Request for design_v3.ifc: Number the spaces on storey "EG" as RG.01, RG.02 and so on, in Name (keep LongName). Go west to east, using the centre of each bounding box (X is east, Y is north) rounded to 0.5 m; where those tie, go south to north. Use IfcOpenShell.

First a look at what the model holds.

```python
import ifcopenshell
import ifcopenshell.util.element
import ifcopenshell.util.placement

model = ifcopenshell.open("design_v3.ifc")
print(model.schema)
storey = next(s for s in model.by_type("IfcBuildingStorey") if s.Name == "EG")
spaces = [e for e in ifcopenshell.util.element.get_decomposition(storey) if e.is_a("IfcSpace")]
for e in sorted(spaces, key=lambda e: e.id()):
    origin = ifcopenshell.util.placement.get_local_placement(e.ObjectPlacement)[:3, 3]
    print(e.id(), e.Name, e.LongName, origin.round(2) + 0.0, sep=" | ")
```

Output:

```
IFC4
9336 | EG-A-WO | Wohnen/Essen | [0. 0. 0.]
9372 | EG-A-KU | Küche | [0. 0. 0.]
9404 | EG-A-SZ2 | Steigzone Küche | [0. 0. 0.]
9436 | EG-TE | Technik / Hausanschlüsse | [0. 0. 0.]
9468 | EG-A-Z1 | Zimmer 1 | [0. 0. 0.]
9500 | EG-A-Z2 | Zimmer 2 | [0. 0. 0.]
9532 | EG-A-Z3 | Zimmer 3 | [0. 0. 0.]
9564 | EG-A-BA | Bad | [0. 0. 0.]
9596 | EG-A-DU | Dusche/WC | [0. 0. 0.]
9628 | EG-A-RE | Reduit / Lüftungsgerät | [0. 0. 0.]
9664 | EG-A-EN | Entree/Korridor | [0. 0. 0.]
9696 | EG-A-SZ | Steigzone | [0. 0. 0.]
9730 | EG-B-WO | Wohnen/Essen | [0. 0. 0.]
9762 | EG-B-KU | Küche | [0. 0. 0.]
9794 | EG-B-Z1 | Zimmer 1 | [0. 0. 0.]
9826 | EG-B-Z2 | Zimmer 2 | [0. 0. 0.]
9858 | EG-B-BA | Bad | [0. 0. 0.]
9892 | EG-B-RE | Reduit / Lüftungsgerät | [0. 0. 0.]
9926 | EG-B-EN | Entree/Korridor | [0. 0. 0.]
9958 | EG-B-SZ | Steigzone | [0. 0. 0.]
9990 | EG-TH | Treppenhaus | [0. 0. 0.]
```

```python
import ifcopenshell
import ifcopenshell.geom
import ifcopenshell.util.element
import ifcopenshell.util.shape

model = ifcopenshell.open("design_v3.ifc")
settings = ifcopenshell.geom.settings()
settings.set("use-world-coords", True)


def centre(element):
    shape = ifcopenshell.geom.create_shape(settings, element)
    return ifcopenshell.util.shape.get_bbox_centroid(shape.geometry)


storey = next(s for s in model.by_type("IfcBuildingStorey") if s.Name == "EG")
spaces = [e for e in ifcopenshell.util.element.get_decomposition(storey) if e.is_a("IfcSpace")]

# Insertion points can sit at a corner or the storey origin, so sort by the geometry (in metres).
centres = {e: centre(e) for e in spaces}
spaces.sort(key=lambda e: (round(centres[e][0] / 0.5), centres[e][1]))

for i, e in enumerate(spaces, start=1):
    number = f"RG.{i:02d}"
    e.Name = number
    print(e.id(), number)

model.write("design_v3_v2.ifc")
```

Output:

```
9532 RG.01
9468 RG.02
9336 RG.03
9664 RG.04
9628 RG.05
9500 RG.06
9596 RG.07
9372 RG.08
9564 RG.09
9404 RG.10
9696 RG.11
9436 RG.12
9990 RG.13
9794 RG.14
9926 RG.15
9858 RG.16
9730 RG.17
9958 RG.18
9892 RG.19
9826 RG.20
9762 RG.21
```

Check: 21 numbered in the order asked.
